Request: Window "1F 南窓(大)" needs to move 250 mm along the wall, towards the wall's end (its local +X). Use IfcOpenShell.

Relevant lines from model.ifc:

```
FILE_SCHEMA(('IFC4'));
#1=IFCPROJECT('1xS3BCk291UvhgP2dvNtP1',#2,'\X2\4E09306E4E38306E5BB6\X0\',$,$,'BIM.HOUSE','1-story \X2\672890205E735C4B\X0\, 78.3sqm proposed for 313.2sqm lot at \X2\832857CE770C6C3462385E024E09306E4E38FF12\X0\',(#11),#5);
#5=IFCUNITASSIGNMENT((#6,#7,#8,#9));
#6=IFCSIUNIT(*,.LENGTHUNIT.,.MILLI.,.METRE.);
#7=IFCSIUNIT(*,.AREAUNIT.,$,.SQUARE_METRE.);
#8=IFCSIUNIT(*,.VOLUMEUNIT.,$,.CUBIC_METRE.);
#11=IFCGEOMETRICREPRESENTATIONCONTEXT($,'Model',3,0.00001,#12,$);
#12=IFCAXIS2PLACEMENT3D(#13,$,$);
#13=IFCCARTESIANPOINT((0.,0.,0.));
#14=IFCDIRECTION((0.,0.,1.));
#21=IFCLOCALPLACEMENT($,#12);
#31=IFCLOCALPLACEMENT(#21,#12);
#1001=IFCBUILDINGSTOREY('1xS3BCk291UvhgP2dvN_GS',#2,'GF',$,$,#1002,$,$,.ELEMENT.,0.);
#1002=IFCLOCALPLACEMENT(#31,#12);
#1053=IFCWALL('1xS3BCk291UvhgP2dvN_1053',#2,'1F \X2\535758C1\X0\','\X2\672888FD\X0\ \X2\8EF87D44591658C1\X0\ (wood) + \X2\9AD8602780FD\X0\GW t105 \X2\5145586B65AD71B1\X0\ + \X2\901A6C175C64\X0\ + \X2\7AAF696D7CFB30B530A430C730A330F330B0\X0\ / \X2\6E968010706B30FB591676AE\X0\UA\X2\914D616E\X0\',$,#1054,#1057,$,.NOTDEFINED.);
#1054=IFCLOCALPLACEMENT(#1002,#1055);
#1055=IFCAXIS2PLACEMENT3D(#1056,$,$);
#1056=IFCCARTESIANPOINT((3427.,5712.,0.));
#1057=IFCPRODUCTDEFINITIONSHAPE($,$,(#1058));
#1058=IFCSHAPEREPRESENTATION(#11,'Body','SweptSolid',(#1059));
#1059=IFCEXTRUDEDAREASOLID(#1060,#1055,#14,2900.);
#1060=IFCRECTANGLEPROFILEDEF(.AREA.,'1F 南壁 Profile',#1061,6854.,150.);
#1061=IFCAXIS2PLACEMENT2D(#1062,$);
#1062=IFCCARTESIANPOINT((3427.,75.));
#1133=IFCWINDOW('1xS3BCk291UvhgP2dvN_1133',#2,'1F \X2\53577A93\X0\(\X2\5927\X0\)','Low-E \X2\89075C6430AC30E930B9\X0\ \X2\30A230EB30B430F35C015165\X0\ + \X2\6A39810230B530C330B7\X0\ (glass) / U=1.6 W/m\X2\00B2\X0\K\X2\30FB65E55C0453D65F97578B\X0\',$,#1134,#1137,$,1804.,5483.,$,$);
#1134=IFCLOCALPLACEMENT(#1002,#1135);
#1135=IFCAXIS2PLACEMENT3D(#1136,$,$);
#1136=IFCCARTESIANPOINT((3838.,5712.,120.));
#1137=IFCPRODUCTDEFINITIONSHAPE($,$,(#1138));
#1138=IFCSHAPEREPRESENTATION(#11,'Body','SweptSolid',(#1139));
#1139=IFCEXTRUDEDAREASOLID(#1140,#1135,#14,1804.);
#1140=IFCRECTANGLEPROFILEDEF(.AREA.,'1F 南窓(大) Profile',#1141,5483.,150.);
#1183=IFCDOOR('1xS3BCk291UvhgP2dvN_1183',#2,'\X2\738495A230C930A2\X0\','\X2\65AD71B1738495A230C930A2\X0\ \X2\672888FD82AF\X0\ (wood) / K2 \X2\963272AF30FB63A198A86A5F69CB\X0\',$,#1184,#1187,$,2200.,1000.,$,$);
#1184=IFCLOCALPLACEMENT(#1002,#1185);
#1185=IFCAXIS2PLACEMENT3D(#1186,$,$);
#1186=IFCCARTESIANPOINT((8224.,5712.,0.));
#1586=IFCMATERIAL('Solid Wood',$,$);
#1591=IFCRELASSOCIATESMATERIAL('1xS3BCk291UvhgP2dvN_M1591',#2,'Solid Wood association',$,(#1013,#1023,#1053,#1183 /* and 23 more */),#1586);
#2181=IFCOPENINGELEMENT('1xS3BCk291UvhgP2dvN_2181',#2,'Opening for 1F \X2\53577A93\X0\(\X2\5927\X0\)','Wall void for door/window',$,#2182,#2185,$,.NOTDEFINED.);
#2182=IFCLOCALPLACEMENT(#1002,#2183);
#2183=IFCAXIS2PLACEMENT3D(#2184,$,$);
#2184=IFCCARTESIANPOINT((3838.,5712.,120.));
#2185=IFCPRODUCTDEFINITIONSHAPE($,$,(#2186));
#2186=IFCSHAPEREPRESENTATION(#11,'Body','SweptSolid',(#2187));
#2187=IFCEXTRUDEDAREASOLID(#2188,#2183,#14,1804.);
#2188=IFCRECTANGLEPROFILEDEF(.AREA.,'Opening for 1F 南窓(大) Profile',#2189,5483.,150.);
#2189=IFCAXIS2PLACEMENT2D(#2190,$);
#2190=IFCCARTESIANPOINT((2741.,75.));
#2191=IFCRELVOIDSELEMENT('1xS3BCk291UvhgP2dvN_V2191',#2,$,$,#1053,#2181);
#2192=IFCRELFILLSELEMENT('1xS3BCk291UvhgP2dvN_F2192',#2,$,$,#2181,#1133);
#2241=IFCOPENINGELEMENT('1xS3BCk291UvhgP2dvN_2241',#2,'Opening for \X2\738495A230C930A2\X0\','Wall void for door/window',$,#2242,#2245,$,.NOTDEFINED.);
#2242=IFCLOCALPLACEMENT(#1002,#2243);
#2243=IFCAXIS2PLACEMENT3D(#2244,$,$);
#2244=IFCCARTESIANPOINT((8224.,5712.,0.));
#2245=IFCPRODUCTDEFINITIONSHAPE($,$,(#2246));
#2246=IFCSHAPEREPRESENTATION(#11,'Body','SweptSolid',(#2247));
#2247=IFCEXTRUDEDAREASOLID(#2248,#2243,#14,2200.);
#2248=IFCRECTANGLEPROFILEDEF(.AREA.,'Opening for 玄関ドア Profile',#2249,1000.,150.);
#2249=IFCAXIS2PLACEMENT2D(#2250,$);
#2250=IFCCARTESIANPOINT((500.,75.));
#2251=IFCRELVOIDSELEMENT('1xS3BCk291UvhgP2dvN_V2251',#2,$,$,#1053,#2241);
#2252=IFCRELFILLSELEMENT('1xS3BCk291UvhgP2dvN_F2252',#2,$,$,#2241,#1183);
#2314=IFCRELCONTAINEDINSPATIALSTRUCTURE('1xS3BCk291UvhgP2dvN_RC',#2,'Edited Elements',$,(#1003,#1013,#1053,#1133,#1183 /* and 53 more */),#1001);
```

```python
import ifcopenshell
import ifcopenshell.api.geometry
import ifcopenshell.util.placement
import ifcopenshell.util.unit

model = ifcopenshell.open("model.ifc")
unit_scale = ifcopenshell.util.unit.calculate_unit_scale(model)

window = model.by_guid("1xS3BCk291UvhgP2dvN_1133")
opening = window.FillsVoids[0].RelatingOpeningElement
wall = opening.VoidsElements[0].RelatingBuildingElement

wall_matrix = ifcopenshell.util.placement.get_local_placement(wall.ObjectPlacement)
shift = wall_matrix[:3, 0] * 0.25 / unit_scale
before = ifcopenshell.util.placement.get_local_placement(window.ObjectPlacement)[:3, 3].copy()

# The window is not placed relative to its opening, so move both.
for product in (opening, window):
    matrix = ifcopenshell.util.placement.get_local_placement(product.ObjectPlacement)
    matrix[:3, 3] += shift
    ifcopenshell.api.geometry.edit_object_placement(model, product=product, matrix=matrix, is_si=False)

after = ifcopenshell.util.placement.get_local_placement(window.ObjectPlacement)[:3, 3]
print("window moved by", (after - before).round(3) + 0.0)

model.write("model-out.ifc")
```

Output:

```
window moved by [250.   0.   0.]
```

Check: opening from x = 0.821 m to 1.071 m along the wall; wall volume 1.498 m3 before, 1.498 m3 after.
